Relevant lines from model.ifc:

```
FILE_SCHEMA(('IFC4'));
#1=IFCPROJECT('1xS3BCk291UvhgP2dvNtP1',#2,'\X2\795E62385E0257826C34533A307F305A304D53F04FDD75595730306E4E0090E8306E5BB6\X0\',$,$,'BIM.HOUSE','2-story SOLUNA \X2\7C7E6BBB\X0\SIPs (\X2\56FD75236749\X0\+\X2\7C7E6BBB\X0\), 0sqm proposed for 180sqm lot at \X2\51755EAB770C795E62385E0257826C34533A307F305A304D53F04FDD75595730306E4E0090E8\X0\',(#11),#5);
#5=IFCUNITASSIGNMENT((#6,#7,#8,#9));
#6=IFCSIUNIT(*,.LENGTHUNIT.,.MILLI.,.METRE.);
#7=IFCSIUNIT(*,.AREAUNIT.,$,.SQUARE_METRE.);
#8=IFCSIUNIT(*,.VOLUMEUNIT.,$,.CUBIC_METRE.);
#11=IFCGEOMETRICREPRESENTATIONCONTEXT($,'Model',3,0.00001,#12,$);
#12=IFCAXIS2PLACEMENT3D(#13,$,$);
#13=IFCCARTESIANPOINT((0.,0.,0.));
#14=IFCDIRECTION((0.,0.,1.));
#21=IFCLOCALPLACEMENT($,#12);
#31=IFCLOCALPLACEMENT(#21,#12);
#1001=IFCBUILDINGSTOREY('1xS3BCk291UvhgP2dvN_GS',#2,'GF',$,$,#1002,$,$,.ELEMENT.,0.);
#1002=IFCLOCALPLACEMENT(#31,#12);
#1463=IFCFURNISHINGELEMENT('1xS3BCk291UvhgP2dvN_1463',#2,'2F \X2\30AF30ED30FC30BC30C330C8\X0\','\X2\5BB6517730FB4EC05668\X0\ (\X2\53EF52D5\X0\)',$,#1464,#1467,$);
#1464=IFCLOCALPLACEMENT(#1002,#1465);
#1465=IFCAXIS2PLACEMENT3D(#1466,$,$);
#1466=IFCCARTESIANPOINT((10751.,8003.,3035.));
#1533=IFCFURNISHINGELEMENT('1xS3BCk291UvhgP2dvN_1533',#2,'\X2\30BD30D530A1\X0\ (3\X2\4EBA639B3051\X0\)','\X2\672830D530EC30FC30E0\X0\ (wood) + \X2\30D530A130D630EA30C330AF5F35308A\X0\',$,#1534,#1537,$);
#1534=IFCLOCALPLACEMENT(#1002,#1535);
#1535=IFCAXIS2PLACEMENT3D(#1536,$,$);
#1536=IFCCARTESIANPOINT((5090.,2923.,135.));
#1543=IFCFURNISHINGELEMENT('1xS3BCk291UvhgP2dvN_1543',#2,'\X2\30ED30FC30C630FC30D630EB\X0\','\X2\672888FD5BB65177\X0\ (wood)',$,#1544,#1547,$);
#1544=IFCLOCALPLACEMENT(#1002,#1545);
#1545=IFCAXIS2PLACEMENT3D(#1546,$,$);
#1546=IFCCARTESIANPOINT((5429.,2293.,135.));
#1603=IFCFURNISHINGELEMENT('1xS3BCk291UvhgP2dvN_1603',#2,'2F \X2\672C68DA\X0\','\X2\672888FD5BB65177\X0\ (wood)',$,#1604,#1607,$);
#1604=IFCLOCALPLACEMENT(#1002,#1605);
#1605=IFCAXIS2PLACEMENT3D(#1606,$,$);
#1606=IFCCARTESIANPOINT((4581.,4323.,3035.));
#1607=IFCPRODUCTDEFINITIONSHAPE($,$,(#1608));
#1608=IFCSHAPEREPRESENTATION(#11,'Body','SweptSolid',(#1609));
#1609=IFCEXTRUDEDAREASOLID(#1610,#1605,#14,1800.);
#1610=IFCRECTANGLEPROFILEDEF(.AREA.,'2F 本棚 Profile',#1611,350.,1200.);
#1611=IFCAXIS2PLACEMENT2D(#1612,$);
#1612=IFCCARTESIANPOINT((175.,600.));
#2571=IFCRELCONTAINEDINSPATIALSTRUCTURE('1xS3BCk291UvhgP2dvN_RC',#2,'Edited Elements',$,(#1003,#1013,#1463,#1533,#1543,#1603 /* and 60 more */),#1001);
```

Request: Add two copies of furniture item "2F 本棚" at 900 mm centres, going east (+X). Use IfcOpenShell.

```python
import numpy as np
import ifcopenshell
import ifcopenshell.api.geometry
import ifcopenshell.api.root
import ifcopenshell.util.element
import ifcopenshell.util.placement
import ifcopenshell.util.unit

model = ifcopenshell.open("model.ifc")
unit_scale = ifcopenshell.util.unit.calculate_unit_scale(model)


def reuse_history(source, copy):
    """copy_class also copies each property set's owner history, people and application; keep the originals."""
    for rel in copy.IsDefinedBy:
        if rel.is_a("IfcRelDefinesByProperties") and (history := rel.RelatingPropertyDefinition.OwnerHistory):
            rel.RelatingPropertyDefinition.OwnerHistory = source.OwnerHistory
            ifcopenshell.util.element.remove_deep2(model, history)


source = model.by_guid("1xS3BCk291UvhgP2dvN_1603")
base = ifcopenshell.util.placement.get_local_placement(source.ObjectPlacement)
step = np.array([1.0, 0.0, 0.0]) * 0.9 / unit_scale

for i in range(1, 3):
    copy = ifcopenshell.api.root.copy_class(model, product=source)
    copy.Representation = ifcopenshell.util.element.copy_deep(
        model, source.Representation, exclude=["IfcGeometricRepresentationContext", "IfcRepresentationMap"]
    )
    reuse_history(source, copy)
    matrix = base.copy()
    matrix[:3, 3] += i * step
    print("added at", matrix[:3, 3].round(3) + 0.0)
    ifcopenshell.api.geometry.edit_object_placement(model, product=copy, matrix=matrix, is_si=False)

model.write("model_rev.ifc")
```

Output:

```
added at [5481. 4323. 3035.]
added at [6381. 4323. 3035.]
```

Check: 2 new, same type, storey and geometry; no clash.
